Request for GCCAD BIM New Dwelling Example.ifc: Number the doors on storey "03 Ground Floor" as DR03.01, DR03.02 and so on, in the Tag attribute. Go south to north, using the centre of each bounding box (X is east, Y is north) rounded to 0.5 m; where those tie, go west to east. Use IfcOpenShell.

First a look at what the model holds.

```python
import ifcopenshell
import ifcopenshell.util.element
import ifcopenshell.util.placement

model = ifcopenshell.open("GCCAD BIM New Dwelling Example.ifc")
print(model.schema)
storey = next(s for s in model.by_type("IfcBuildingStorey") if s.Name == "03 Ground Floor")
doors = [e for e in ifcopenshell.util.element.get_decomposition(storey) if e.is_a("IfcDoor")]
for e in sorted(doors, key=lambda e: e.id()):
    origin = ifcopenshell.util.placement.get_local_placement(e.ObjectPlacement)[:3, 3]
    print(e.id(), e.Tag, e.Name, origin.round(2) + 0.0, sep=" | ")
```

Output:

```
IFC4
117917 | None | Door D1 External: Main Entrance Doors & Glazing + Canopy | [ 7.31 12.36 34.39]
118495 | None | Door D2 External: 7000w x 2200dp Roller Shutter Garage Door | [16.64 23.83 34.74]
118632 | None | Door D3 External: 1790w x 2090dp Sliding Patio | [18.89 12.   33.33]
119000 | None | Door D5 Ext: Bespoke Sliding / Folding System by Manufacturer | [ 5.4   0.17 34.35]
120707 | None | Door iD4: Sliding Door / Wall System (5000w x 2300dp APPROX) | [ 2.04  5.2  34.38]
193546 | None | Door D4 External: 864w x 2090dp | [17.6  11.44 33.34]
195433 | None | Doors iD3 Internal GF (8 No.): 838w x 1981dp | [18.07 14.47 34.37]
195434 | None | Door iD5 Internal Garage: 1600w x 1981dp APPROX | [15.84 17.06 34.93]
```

```python
import ifcopenshell
import ifcopenshell.geom
import ifcopenshell.util.element
import ifcopenshell.util.shape

model = ifcopenshell.open("GCCAD BIM New Dwelling Example.ifc")
settings = ifcopenshell.geom.settings()
settings.set("use-world-coords", True)


def centre(element):
    shape = ifcopenshell.geom.create_shape(settings, element)
    return ifcopenshell.util.shape.get_bbox_centroid(shape.geometry)


storey = next(s for s in model.by_type("IfcBuildingStorey") if s.Name == "03 Ground Floor")
doors = [e for e in ifcopenshell.util.element.get_decomposition(storey) if e.is_a("IfcDoor")]

# Insertion points can sit at a corner or the storey origin, so sort by the geometry (in metres).
centres = {e: centre(e) for e in doors}
doors.sort(key=lambda e: (round(centres[e][1] / 0.5), centres[e][0]))

for i, e in enumerate(doors, start=1):
    number = f"DR03.{i:02d}"
    e.Tag = number
    print(e.id(), number)

model.write("GCCAD BIM New Dwelling Example-out.ifc")
```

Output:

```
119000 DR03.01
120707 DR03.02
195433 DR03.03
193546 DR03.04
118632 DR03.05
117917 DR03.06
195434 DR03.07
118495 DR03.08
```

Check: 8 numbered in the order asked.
